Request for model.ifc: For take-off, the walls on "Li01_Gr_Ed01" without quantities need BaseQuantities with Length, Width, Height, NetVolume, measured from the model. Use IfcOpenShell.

First a look at what the model holds.

```python
import ifcopenshell
import ifcopenshell.util.element
import ifcopenshell.util.unit

model = ifcopenshell.open("model.ifc")
print(model.schema)
for unit_type in ("LENGTHUNIT", "AREAUNIT", "VOLUMEUNIT"):
    print(unit_type, ifcopenshell.util.unit.calculate_unit_scale(model, unit_type))
storey = next(s for s in model.by_type("IfcBuildingStorey") if s.Name == "Li01_Gr_Ed01")
walls = [e for e in ifcopenshell.util.element.get_decomposition(storey) if e.is_a("IfcWall")]
for e in sorted(walls, key=lambda e: e.id()):
    print(e.id(), e.is_a(), e.Name, list(ifcopenshell.util.element.get_psets(e, qtos_only=True)), sep=" | ")
```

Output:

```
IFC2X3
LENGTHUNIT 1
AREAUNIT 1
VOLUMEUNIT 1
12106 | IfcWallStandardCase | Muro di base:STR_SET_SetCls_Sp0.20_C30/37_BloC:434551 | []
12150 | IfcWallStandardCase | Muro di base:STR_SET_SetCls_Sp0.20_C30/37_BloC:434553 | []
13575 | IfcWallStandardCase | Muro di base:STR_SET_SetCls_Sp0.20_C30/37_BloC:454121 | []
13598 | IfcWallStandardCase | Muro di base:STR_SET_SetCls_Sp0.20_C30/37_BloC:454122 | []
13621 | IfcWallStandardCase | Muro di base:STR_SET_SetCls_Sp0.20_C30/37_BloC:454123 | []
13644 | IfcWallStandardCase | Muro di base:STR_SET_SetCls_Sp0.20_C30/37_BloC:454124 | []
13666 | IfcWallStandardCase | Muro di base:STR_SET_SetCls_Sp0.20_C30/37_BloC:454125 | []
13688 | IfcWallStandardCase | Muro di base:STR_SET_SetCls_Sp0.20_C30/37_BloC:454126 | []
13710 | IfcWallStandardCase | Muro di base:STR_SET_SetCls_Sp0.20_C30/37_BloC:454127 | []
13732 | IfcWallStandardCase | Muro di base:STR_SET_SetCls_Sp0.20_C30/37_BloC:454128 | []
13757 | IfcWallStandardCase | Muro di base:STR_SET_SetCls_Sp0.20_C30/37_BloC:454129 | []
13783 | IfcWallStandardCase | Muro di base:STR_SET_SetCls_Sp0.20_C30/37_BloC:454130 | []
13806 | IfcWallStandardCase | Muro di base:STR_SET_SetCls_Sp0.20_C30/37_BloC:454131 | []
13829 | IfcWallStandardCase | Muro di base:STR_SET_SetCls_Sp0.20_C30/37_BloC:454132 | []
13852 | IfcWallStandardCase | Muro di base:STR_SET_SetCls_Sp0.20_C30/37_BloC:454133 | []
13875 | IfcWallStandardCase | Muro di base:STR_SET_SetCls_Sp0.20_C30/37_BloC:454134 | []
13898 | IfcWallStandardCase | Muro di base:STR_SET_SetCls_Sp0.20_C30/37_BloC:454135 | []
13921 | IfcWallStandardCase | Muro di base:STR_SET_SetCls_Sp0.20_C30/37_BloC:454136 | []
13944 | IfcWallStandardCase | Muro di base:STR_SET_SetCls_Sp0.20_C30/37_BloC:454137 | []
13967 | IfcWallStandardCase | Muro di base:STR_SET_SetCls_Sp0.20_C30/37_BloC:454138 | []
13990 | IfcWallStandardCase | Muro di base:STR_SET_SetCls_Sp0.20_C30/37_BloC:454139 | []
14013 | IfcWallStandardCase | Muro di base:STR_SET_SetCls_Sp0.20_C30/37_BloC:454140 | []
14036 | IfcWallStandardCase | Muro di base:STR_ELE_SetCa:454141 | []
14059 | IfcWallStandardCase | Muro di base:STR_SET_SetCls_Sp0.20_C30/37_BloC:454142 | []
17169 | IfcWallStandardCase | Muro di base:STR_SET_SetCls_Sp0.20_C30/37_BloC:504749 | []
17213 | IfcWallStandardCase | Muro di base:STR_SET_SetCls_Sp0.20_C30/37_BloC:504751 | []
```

```python
import ifcopenshell
import ifcopenshell.api.pset
import ifcopenshell.geom
import ifcopenshell.util.element
import ifcopenshell.util.shape
import ifcopenshell.util.unit

model = ifcopenshell.open("model.ifc")
unit_scale = ifcopenshell.util.unit.calculate_unit_scale(model)
volume_scale = ifcopenshell.util.unit.calculate_unit_scale(model, "VOLUMEUNIT")
settings = ifcopenshell.geom.settings()

storey = next(s for s in model.by_type("IfcBuildingStorey") if s.Name == "Li01_Gr_Ed01")
walls = [e for e in ifcopenshell.util.element.get_decomposition(storey) if e.is_a("IfcWall")]

for e in sorted(walls, key=lambda e: e.id()):
    if ifcopenshell.util.element.get_psets(e, qtos_only=True, should_inherit=False):
        continue
    # Geometry comes back in metres, in the element's own axes.
    shape = ifcopenshell.geom.create_shape(settings, e)
    values = {
        "Length": ifcopenshell.util.shape.get_x(shape.geometry) / unit_scale,
        "Width": ifcopenshell.util.shape.get_y(shape.geometry) / unit_scale,
        "Height": ifcopenshell.util.shape.get_z(shape.geometry) / unit_scale,
        "NetVolume": ifcopenshell.util.shape.get_volume(shape.geometry) / volume_scale,
    }
    qto = ifcopenshell.api.pset.add_qto(model, product=e, name="BaseQuantities")
    ifcopenshell.api.pset.edit_qto(model, qto=qto, properties=values)
    print(e.id(), {k: round(v, 3) for k, v in values.items()})

model.write("model_v2.ifc")
```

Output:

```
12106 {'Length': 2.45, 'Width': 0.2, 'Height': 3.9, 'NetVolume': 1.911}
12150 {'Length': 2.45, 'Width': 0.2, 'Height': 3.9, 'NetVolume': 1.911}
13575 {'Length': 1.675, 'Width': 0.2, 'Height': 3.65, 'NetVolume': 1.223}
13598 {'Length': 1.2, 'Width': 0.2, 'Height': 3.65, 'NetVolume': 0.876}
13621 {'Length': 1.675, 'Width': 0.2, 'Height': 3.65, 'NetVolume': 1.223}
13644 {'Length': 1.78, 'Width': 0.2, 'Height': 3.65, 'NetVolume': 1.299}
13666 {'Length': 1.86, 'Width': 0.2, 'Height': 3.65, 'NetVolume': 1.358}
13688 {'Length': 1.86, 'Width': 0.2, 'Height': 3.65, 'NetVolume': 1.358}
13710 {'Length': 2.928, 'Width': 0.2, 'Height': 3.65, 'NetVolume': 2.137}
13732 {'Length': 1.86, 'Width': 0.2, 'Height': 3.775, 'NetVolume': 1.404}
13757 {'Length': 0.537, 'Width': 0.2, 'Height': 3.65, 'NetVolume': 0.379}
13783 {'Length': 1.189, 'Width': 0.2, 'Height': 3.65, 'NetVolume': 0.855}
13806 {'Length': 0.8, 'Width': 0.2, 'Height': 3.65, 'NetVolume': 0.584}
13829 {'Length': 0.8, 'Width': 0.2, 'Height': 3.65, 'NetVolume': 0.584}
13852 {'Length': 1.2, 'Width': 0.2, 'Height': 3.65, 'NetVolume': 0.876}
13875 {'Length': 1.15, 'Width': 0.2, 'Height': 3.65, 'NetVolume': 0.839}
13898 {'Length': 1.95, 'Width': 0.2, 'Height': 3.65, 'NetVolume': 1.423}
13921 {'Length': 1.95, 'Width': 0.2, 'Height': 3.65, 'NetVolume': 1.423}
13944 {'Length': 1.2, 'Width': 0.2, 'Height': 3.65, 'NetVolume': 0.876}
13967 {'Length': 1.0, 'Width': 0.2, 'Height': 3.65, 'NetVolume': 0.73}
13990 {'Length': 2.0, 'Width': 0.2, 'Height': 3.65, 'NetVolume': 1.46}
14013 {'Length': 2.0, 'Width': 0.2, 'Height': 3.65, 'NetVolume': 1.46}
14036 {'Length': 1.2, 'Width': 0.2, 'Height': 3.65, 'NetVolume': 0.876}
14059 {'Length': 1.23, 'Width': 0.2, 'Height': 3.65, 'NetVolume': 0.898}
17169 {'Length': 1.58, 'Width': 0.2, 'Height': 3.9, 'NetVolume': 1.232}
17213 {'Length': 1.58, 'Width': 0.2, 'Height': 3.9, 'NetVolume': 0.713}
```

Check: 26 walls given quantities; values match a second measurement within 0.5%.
